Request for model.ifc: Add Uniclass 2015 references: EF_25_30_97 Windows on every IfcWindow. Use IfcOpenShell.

First a look at what the model holds.

```python
import ifcopenshell

model = ifcopenshell.open("model.ifc")
print(model.schema)
print("classifications:", [c.Name for c in model.by_type("IfcClassification")])
for ifc_class in ("IfcDoor", "IfcRoof", "IfcStair", "IfcWall", "IfcWindow"):
    print(ifc_class, len(model.by_type(ifc_class)))
```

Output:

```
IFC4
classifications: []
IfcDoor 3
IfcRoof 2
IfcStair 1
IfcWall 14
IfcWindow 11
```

```python
import ifcopenshell
import ifcopenshell.api.classification

model = ifcopenshell.open("model.ifc")

system = ifcopenshell.api.classification.add_classification(model, classification="Uniclass 2015")

codes = {
    "IfcWindow": ("EF_25_30_97", "Windows"),
}
for ifc_class, (code, name) in codes.items():
    products = model.by_type(ifc_class)
    ifcopenshell.api.classification.add_reference(
        model, products=products, classification=system, identification=code, name=name
    )
    print(code, len(products))

model.write("model_edited.ifc")
```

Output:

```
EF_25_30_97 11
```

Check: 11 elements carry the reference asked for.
